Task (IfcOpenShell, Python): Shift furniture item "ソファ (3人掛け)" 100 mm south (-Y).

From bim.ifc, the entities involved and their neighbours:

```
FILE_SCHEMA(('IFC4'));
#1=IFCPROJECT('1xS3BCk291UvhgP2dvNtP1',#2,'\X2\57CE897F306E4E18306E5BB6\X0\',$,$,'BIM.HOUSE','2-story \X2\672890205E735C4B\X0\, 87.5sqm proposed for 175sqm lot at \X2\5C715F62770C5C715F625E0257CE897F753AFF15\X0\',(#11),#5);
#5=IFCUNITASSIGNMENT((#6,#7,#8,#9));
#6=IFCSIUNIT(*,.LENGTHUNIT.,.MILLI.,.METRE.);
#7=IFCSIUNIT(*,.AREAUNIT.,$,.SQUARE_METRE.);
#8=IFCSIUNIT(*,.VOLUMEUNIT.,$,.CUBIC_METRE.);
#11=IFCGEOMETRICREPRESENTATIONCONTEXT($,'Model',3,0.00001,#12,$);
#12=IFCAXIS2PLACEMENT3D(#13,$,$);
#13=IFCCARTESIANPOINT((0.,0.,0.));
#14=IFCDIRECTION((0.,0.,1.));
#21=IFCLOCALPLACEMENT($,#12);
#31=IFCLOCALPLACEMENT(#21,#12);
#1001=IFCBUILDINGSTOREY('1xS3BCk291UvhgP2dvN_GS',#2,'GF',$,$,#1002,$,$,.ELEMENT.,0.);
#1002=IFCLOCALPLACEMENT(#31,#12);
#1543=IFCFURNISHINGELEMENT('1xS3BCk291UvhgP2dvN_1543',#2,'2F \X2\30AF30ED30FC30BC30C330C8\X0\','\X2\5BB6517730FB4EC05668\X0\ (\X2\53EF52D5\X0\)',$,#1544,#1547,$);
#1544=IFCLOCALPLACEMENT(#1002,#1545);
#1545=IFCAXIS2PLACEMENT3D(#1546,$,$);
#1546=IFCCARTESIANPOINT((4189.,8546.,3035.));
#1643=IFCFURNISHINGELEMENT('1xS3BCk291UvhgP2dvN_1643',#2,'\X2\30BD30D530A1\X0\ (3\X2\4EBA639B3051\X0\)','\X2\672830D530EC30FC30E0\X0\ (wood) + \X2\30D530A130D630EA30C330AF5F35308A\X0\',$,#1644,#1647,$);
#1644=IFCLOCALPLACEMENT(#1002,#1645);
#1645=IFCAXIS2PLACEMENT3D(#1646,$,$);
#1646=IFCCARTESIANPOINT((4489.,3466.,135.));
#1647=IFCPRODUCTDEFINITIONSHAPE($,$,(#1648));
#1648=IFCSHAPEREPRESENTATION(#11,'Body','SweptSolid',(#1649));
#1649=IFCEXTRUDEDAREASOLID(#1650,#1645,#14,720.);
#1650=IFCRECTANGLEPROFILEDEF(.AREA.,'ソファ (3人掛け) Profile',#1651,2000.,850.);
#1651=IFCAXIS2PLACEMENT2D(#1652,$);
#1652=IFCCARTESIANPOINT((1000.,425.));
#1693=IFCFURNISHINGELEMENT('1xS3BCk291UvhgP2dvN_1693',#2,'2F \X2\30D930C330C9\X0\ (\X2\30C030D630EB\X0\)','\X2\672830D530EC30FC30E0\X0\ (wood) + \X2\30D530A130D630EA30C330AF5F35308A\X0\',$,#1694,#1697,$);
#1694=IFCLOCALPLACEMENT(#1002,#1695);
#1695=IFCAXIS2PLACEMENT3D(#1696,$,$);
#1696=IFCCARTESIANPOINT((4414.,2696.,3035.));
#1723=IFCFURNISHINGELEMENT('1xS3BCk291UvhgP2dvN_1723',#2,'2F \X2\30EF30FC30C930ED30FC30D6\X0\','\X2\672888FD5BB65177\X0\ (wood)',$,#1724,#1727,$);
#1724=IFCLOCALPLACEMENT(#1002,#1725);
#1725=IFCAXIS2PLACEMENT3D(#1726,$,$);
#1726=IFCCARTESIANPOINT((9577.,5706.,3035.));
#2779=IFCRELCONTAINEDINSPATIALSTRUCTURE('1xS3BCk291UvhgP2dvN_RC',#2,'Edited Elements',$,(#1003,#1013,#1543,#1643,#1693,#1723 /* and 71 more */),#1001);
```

```python
import ifcopenshell
import ifcopenshell.api.geometry
import ifcopenshell.util.placement

model = ifcopenshell.open("bim.ifc")

item = model.by_guid("1xS3BCk291UvhgP2dvN_1643")
matrix = ifcopenshell.util.placement.get_local_placement(item.ObjectPlacement)
matrix[1, 3] -= 100.0
ifcopenshell.api.geometry.edit_object_placement(model, product=item, matrix=matrix, is_si=False)

print(ifcopenshell.util.placement.get_local_placement(item.ObjectPlacement).round(3) + 0.0)

model.write("bim_updated.ifc")
```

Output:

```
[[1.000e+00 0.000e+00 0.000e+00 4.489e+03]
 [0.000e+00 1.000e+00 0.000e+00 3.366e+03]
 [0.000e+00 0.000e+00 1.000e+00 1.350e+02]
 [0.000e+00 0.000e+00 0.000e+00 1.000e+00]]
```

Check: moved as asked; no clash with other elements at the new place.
